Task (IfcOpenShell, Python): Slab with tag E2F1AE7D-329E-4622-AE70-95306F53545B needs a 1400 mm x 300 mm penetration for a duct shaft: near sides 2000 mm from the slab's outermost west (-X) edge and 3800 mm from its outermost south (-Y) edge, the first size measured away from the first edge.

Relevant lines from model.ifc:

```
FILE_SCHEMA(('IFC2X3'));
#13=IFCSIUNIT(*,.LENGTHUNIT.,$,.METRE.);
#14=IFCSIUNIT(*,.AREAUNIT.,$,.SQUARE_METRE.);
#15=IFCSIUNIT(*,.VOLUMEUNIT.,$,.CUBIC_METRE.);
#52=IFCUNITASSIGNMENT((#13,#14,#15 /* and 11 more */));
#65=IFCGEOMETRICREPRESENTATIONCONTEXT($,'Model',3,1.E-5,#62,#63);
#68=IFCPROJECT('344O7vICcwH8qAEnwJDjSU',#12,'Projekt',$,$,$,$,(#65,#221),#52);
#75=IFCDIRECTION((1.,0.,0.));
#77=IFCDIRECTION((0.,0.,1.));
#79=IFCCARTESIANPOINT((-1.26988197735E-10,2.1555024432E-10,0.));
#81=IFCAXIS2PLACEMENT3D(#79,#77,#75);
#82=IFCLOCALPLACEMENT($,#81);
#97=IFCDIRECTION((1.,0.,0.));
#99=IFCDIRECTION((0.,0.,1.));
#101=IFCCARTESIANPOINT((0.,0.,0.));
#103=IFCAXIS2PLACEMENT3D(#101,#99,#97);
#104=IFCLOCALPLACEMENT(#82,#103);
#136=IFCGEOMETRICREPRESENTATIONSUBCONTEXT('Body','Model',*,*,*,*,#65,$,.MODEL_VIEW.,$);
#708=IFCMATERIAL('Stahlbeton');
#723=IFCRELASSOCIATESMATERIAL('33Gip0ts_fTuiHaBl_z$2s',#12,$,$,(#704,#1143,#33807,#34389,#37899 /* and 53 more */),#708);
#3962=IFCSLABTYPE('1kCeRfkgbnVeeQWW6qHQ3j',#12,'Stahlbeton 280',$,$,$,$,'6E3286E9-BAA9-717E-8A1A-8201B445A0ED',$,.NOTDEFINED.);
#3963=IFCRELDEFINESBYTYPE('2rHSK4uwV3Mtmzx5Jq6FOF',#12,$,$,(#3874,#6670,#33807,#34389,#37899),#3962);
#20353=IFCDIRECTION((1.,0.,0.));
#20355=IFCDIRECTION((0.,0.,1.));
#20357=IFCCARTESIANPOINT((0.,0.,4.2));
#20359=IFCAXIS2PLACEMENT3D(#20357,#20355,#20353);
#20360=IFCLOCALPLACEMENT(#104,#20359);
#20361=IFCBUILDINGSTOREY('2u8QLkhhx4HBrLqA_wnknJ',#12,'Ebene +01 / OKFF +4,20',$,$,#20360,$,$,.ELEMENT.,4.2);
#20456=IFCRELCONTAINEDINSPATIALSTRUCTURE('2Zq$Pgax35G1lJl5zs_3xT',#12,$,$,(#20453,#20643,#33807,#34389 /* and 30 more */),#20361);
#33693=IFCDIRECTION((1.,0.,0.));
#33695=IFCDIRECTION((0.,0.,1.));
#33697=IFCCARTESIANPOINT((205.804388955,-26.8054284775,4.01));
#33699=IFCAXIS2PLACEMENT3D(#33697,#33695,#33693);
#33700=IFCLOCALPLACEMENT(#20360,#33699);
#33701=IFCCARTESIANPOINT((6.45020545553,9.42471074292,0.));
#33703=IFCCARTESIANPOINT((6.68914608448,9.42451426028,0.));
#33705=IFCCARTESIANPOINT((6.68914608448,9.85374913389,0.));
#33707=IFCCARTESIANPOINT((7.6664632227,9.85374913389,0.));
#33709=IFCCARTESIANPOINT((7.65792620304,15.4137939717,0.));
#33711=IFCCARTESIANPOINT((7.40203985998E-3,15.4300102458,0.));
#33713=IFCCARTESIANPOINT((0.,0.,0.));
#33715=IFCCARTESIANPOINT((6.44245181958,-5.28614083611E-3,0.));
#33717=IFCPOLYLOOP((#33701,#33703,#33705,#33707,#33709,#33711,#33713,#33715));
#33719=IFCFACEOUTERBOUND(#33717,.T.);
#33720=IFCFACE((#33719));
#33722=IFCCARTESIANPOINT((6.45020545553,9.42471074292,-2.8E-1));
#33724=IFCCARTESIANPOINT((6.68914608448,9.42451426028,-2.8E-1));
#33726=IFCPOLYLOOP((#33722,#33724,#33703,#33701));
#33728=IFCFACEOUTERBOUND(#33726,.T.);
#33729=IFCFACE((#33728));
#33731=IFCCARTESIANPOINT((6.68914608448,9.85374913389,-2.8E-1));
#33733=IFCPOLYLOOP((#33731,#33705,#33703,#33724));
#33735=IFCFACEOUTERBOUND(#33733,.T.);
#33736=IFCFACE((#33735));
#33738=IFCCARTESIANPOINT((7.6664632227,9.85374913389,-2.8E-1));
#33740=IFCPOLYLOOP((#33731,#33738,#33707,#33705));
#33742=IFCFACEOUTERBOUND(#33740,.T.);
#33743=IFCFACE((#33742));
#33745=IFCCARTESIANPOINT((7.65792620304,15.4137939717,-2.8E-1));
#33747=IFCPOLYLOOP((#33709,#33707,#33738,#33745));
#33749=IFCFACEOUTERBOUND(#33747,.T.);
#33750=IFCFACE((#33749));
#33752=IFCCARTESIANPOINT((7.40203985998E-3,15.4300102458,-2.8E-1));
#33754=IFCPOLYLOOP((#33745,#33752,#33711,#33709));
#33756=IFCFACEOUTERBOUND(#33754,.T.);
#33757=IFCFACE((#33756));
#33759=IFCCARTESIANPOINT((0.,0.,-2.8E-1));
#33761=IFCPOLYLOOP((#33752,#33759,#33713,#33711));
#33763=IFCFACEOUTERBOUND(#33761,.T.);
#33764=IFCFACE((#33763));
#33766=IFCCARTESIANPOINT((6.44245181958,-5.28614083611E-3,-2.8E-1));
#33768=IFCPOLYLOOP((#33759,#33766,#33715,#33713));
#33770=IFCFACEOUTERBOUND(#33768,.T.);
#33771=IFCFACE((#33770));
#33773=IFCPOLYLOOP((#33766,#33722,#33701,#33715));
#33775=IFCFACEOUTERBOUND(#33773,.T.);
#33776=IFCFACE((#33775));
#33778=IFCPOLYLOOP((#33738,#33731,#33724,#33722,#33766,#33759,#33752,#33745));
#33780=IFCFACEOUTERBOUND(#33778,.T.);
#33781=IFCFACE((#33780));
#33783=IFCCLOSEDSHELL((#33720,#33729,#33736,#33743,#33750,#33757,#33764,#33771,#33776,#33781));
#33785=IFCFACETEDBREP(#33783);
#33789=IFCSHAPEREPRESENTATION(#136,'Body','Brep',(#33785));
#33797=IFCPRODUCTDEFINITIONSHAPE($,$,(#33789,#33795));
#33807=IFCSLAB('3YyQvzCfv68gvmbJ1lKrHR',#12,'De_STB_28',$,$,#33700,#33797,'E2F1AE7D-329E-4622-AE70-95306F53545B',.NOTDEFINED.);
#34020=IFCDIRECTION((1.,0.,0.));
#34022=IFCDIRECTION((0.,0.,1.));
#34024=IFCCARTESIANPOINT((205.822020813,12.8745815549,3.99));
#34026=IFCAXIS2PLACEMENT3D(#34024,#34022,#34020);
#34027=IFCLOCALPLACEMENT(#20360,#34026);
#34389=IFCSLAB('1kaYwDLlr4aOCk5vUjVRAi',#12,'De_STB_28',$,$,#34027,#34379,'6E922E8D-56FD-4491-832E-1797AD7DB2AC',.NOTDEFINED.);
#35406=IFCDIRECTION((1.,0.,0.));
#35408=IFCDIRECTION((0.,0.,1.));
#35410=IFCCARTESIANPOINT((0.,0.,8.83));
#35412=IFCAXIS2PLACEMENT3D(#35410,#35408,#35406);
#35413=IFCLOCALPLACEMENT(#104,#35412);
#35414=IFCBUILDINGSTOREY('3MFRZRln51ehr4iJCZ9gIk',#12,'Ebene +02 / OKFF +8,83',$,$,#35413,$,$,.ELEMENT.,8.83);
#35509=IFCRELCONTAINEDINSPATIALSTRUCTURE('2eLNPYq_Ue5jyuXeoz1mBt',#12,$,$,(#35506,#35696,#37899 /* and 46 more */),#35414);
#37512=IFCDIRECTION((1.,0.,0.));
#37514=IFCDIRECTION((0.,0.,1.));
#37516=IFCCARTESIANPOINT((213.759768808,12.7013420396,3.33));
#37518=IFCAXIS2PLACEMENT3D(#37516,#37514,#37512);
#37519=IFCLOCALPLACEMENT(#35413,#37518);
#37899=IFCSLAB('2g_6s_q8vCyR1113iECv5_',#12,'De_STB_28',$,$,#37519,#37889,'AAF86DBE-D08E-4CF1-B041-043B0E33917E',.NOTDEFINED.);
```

```python
import numpy as np
import ifcopenshell
import ifcopenshell.api.feature
import ifcopenshell.api.geometry
import ifcopenshell.api.root
import ifcopenshell.geom
import ifcopenshell.util.placement
import ifcopenshell.util.representation
import ifcopenshell.util.shape
import ifcopenshell.util.unit

model = ifcopenshell.open("model.ifc")
unit_scale = ifcopenshell.util.unit.calculate_unit_scale(model)
settings = ifcopenshell.geom.settings()


def volume(element):
    """Net volume in cubic metres, openings subtracted."""
    shape = ifcopenshell.geom.create_shape(settings, element)
    return ifcopenshell.util.shape.get_volume(shape.geometry)


slab = model.by_id(33807)
before = volume(slab)

# Extent in the slab's own axes, in metres. The edges named are its -X and -Y sides.
slab_shape = ifcopenshell.geom.create_shape(settings, slab)
vertices = ifcopenshell.util.shape.get_vertices(slab_shape.geometry)
x_min, y_min, bottom = vertices.min(axis=0)
top = vertices[:, 2].max()

opening = ifcopenshell.api.root.create_entity(model, ifc_class="IfcOpeningElement", name="Duct shaft opening")
context = ifcopenshell.util.representation.get_context(model, "Model", "Body", "MODEL_VIEW")
width, depth = 1.4, 0.3
outline = [(0.0, 0.0), (width, 0.0), (width, depth), (0.0, depth), (0.0, 0.0)]
# Overshoot both faces by 50 mm so the cut is clean.
shape = ifcopenshell.api.geometry.add_slab_representation(
    model, context=context, depth=top - bottom + 0.1, polyline=outline
)
ifcopenshell.api.geometry.assign_representation(model, product=opening, representation=shape)

matrix = ifcopenshell.util.placement.get_local_placement(slab.ObjectPlacement)
matrix[:, 3] = matrix @ np.append(np.array([x_min + 2, y_min + 3.8, bottom - 0.05]) / unit_scale, 1.0)
ifcopenshell.api.geometry.edit_object_placement(model, product=opening, matrix=matrix, is_si=False)
ifcopenshell.api.feature.add_feature(model, feature=opening, element=slab)

after = volume(slab)

print(f"slab volume {before:.3f} -> {after:.3f} m3")

model.write("model_v2.ifc")
```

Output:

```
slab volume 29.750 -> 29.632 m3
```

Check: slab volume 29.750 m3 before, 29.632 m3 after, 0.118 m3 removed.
